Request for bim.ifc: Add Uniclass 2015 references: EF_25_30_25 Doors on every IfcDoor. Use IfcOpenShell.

First a look at what the model holds.

```python
import ifcopenshell

model = ifcopenshell.open("bim.ifc")
print(model.schema)
print("classifications:", [c.Name for c in model.by_type("IfcClassification")])
for ifc_class in ("IfcDoor", "IfcRoof", "IfcStair", "IfcWall", "IfcWindow"):
    print(ifc_class, len(model.by_type(ifc_class)))
```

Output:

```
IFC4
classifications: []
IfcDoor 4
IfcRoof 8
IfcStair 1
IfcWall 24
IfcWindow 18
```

```python
import ifcopenshell
import ifcopenshell.api.classification

model = ifcopenshell.open("bim.ifc")

system = ifcopenshell.api.classification.add_classification(model, classification="Uniclass 2015")

codes = {
    "IfcDoor": ("EF_25_30_25", "Doors"),
}
for ifc_class, (code, name) in codes.items():
    products = model.by_type(ifc_class)
    ifcopenshell.api.classification.add_reference(
        model, products=products, classification=system, identification=code, name=name
    )
    print(code, len(products))

model.write("bim-out.ifc")
```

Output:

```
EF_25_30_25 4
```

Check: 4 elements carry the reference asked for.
